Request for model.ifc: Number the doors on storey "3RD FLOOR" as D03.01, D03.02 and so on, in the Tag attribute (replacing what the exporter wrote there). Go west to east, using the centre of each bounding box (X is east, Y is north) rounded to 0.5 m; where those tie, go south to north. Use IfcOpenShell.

First a look at what the model holds.

```python
import ifcopenshell
import ifcopenshell.util.element
import ifcopenshell.util.placement

model = ifcopenshell.open("model.ifc")
print(model.schema)
storey = next(s for s in model.by_type("IfcBuildingStorey") if s.Name == "3RD FLOOR")
doors = [e for e in ifcopenshell.util.element.get_decomposition(storey) if e.is_a("IfcDoor")]
for e in sorted(doors, key=lambda e: e.id()):
    origin = ifcopenshell.util.placement.get_local_placement(e.ObjectPlacement)[:3, 3]
    print(e.id(), e.Tag, e.Name, origin.round(2) + 0.0, sep=" | ")
```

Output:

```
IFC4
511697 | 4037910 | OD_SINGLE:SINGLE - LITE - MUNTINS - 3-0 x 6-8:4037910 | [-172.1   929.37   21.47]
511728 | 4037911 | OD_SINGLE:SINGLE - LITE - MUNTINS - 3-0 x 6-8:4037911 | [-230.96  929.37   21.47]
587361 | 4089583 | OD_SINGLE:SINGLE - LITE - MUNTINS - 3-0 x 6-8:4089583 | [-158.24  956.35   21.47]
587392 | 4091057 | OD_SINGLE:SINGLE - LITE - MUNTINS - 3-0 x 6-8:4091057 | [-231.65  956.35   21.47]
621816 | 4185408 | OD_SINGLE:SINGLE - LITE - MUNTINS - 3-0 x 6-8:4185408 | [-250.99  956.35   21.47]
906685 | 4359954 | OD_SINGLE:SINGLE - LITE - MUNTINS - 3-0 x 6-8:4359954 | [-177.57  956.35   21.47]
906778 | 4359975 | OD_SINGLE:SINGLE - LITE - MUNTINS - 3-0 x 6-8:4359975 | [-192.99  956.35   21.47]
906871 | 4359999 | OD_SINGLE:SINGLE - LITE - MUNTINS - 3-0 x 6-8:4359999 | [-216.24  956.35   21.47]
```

```python
import ifcopenshell
import ifcopenshell.geom
import ifcopenshell.util.element
import ifcopenshell.util.shape

model = ifcopenshell.open("model.ifc")
settings = ifcopenshell.geom.settings()
settings.set("use-world-coords", True)


def centre(element):
    shape = ifcopenshell.geom.create_shape(settings, element)
    return ifcopenshell.util.shape.get_bbox_centroid(shape.geometry)


storey = next(s for s in model.by_type("IfcBuildingStorey") if s.Name == "3RD FLOOR")
doors = [e for e in ifcopenshell.util.element.get_decomposition(storey) if e.is_a("IfcDoor")]

# Insertion points can sit at a corner or the storey origin, so sort by the geometry (in metres).
centres = {e: centre(e) for e in doors}
doors.sort(key=lambda e: (round(centres[e][0] / 0.5), centres[e][1]))

for i, e in enumerate(doors, start=1):
    number = f"D03.{i:02d}"
    e.Tag = number
    print(e.id(), number)

model.write("model_updated.ifc")
```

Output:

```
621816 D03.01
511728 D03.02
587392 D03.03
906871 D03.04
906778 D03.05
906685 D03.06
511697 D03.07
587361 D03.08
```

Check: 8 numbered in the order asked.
